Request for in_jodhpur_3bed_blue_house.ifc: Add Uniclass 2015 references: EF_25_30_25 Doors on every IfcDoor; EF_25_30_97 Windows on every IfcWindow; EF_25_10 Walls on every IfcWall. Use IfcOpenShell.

First a look at what the model holds.

```python
import ifcopenshell

model = ifcopenshell.open("in_jodhpur_3bed_blue_house.ifc")
print(model.schema)
print("classifications:", [c.Name for c in model.by_type("IfcClassification")])
for ifc_class in ("IfcDoor", "IfcRoof", "IfcStair", "IfcWall", "IfcWindow"):
    print(ifc_class, len(model.by_type(ifc_class)))
```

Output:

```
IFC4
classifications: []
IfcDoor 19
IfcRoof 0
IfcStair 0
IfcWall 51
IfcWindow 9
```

```python
import ifcopenshell
import ifcopenshell.api.classification

model = ifcopenshell.open("in_jodhpur_3bed_blue_house.ifc")

system = ifcopenshell.api.classification.add_classification(model, classification="Uniclass 2015")

codes = {
    "IfcDoor": ("EF_25_30_25", "Doors"),
    "IfcWindow": ("EF_25_30_97", "Windows"),
    "IfcWall": ("EF_25_10", "Walls"),
}
for ifc_class, (code, name) in codes.items():
    products = model.by_type(ifc_class)
    ifcopenshell.api.classification.add_reference(
        model, products=products, classification=system, identification=code, name=name
    )
    print(code, len(products))

model.write("in_jodhpur_3bed_blue_house_updated.ifc")
```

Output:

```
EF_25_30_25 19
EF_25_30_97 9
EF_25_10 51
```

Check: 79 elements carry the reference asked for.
